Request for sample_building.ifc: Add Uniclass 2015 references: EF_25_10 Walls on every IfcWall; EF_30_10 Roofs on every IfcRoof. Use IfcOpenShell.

First a look at what the model holds.

```python
import ifcopenshell

model = ifcopenshell.open("sample_building.ifc")
print(model.schema)
print("classifications:", [c.Name for c in model.by_type("IfcClassification")])
for ifc_class in ("IfcDoor", "IfcRoof", "IfcStair", "IfcWall", "IfcWindow"):
    print(ifc_class, len(model.by_type(ifc_class)))
```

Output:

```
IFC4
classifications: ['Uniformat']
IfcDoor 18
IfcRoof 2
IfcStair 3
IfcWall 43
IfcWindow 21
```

```python
import ifcopenshell
import ifcopenshell.api.classification

model = ifcopenshell.open("sample_building.ifc")

system = ifcopenshell.api.classification.add_classification(model, classification="Uniclass 2015")

codes = {
    "IfcWall": ("EF_25_10", "Walls"),
    "IfcRoof": ("EF_30_10", "Roofs"),
}
for ifc_class, (code, name) in codes.items():
    products = model.by_type(ifc_class)
    ifcopenshell.api.classification.add_reference(
        model, products=products, classification=system, identification=code, name=name
    )
    print(code, len(products))

model.write("sample_building_rev.ifc")
```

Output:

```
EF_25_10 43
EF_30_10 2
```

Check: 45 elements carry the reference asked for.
